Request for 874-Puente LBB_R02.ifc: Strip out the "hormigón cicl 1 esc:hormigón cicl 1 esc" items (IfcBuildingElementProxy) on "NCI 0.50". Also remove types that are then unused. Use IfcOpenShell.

First a look at what the model holds.

```python
import ifcopenshell
import ifcopenshell.util.element

model = ifcopenshell.open("874-Puente LBB_R02.ifc")
print(model.schema)
storey = next(s for s in model.by_type("IfcBuildingStorey") if s.Name == "NCI 0.50")
proxies = [e for e in ifcopenshell.util.element.get_decomposition(storey) if e.is_a("IfcBuildingElementProxy")]
seen = {}
for e in proxies:
    element_type = ifcopenshell.util.element.get_type(e)
    name = element_type.Name if element_type not in (None, e) else None
    seen[name] = seen.get(name, 0) + 1
for name, count in sorted(seen.items(), key=str):
    print(count, "x", name)
```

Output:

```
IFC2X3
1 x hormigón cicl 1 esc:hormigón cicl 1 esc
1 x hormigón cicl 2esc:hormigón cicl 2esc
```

```python
import ifcopenshell
import ifcopenshell.api.root
import ifcopenshell.util.element

model = ifcopenshell.open("874-Puente LBB_R02.ifc")

storey = next(s for s in model.by_type("IfcBuildingStorey") if s.Name == "NCI 0.50")
proxies = [e for e in ifcopenshell.util.element.get_decomposition(storey) if e.is_a("IfcBuildingElementProxy")]
targets = [e for e in proxies if (t := ifcopenshell.util.element.get_type(e)) not in (None, e) and t.Name == "hormigón cicl 1 esc:hormigón cicl 1 esc"]
types = {ifcopenshell.util.element.get_type(e) for e in targets} - {None, *targets}

for e in targets:
    ifcopenshell.api.root.remove_product(model, product=e)
print(len(targets), "removed")

unused = [t for t in types if not ifcopenshell.util.element.get_types(t)]
for t in unused:
    ifcopenshell.api.root.remove_product(model, product=t)
print(len(unused), "unused types removed")

model.write("874-Puente LBB_R02_v2.ifc")
```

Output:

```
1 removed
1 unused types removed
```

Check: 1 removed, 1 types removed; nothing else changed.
